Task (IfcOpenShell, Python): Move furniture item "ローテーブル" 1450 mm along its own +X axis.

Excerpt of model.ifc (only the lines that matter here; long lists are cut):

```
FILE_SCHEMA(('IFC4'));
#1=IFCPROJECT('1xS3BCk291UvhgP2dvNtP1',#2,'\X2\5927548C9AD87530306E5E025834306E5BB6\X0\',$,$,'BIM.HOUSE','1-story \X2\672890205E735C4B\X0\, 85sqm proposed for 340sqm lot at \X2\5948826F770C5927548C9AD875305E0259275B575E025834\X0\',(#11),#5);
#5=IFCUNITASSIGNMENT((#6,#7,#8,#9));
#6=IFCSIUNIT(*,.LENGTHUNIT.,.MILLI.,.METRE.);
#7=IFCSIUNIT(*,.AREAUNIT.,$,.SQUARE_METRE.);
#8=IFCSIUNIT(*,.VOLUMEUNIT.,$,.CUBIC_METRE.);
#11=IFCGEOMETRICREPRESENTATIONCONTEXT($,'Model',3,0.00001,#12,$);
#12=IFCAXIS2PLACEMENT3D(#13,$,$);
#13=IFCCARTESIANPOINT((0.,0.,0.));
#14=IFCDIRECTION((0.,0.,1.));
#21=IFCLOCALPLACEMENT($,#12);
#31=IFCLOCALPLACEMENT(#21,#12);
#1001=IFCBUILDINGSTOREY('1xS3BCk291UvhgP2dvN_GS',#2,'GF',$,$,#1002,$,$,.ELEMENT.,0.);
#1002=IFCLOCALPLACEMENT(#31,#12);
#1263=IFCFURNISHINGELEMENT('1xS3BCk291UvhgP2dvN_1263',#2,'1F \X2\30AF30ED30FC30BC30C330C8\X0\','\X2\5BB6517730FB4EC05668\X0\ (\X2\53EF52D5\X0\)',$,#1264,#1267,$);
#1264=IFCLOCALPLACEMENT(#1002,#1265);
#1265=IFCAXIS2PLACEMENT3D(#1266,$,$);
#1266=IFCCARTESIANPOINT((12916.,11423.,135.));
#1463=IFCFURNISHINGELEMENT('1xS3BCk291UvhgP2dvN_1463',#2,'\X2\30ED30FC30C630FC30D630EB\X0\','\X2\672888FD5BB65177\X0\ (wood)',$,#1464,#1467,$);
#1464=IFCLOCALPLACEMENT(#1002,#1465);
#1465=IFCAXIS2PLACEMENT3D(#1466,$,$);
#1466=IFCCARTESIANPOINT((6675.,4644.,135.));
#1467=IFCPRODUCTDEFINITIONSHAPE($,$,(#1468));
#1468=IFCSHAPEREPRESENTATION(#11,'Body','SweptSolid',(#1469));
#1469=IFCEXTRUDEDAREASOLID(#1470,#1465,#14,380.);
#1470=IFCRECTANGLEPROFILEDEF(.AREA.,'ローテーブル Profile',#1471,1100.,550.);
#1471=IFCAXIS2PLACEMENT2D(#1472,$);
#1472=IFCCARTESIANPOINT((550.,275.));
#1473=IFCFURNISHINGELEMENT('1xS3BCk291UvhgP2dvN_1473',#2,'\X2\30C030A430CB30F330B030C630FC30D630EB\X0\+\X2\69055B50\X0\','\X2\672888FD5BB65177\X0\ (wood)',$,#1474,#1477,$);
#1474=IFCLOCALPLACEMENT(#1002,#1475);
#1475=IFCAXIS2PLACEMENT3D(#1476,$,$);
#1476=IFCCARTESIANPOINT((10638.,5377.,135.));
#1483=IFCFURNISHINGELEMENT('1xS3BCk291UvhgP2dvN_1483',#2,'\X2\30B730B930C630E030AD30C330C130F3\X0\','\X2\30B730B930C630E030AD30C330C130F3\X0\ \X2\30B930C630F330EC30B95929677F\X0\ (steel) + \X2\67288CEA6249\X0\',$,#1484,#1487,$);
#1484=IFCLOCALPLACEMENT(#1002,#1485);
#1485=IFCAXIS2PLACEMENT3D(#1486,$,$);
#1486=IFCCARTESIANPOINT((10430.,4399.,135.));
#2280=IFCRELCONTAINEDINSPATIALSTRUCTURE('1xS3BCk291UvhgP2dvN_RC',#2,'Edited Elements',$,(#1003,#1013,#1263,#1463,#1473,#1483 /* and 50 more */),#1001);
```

```python
import ifcopenshell
import ifcopenshell.api.geometry
import ifcopenshell.util.placement

model = ifcopenshell.open("model.ifc")

item = model.by_guid("1xS3BCk291UvhgP2dvN_1463")
matrix = ifcopenshell.util.placement.get_local_placement(item.ObjectPlacement)
matrix[:3, 3] += matrix[:3, 0] * 1450.0
ifcopenshell.api.geometry.edit_object_placement(model, product=item, matrix=matrix, is_si=False)

print(ifcopenshell.util.placement.get_local_placement(item.ObjectPlacement).round(3) + 0.0)

model.write("model-out.ifc")
```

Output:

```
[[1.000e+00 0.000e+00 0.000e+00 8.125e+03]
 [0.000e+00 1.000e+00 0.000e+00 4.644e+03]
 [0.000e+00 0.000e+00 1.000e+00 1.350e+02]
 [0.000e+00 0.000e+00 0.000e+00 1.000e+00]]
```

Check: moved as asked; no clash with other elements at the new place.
